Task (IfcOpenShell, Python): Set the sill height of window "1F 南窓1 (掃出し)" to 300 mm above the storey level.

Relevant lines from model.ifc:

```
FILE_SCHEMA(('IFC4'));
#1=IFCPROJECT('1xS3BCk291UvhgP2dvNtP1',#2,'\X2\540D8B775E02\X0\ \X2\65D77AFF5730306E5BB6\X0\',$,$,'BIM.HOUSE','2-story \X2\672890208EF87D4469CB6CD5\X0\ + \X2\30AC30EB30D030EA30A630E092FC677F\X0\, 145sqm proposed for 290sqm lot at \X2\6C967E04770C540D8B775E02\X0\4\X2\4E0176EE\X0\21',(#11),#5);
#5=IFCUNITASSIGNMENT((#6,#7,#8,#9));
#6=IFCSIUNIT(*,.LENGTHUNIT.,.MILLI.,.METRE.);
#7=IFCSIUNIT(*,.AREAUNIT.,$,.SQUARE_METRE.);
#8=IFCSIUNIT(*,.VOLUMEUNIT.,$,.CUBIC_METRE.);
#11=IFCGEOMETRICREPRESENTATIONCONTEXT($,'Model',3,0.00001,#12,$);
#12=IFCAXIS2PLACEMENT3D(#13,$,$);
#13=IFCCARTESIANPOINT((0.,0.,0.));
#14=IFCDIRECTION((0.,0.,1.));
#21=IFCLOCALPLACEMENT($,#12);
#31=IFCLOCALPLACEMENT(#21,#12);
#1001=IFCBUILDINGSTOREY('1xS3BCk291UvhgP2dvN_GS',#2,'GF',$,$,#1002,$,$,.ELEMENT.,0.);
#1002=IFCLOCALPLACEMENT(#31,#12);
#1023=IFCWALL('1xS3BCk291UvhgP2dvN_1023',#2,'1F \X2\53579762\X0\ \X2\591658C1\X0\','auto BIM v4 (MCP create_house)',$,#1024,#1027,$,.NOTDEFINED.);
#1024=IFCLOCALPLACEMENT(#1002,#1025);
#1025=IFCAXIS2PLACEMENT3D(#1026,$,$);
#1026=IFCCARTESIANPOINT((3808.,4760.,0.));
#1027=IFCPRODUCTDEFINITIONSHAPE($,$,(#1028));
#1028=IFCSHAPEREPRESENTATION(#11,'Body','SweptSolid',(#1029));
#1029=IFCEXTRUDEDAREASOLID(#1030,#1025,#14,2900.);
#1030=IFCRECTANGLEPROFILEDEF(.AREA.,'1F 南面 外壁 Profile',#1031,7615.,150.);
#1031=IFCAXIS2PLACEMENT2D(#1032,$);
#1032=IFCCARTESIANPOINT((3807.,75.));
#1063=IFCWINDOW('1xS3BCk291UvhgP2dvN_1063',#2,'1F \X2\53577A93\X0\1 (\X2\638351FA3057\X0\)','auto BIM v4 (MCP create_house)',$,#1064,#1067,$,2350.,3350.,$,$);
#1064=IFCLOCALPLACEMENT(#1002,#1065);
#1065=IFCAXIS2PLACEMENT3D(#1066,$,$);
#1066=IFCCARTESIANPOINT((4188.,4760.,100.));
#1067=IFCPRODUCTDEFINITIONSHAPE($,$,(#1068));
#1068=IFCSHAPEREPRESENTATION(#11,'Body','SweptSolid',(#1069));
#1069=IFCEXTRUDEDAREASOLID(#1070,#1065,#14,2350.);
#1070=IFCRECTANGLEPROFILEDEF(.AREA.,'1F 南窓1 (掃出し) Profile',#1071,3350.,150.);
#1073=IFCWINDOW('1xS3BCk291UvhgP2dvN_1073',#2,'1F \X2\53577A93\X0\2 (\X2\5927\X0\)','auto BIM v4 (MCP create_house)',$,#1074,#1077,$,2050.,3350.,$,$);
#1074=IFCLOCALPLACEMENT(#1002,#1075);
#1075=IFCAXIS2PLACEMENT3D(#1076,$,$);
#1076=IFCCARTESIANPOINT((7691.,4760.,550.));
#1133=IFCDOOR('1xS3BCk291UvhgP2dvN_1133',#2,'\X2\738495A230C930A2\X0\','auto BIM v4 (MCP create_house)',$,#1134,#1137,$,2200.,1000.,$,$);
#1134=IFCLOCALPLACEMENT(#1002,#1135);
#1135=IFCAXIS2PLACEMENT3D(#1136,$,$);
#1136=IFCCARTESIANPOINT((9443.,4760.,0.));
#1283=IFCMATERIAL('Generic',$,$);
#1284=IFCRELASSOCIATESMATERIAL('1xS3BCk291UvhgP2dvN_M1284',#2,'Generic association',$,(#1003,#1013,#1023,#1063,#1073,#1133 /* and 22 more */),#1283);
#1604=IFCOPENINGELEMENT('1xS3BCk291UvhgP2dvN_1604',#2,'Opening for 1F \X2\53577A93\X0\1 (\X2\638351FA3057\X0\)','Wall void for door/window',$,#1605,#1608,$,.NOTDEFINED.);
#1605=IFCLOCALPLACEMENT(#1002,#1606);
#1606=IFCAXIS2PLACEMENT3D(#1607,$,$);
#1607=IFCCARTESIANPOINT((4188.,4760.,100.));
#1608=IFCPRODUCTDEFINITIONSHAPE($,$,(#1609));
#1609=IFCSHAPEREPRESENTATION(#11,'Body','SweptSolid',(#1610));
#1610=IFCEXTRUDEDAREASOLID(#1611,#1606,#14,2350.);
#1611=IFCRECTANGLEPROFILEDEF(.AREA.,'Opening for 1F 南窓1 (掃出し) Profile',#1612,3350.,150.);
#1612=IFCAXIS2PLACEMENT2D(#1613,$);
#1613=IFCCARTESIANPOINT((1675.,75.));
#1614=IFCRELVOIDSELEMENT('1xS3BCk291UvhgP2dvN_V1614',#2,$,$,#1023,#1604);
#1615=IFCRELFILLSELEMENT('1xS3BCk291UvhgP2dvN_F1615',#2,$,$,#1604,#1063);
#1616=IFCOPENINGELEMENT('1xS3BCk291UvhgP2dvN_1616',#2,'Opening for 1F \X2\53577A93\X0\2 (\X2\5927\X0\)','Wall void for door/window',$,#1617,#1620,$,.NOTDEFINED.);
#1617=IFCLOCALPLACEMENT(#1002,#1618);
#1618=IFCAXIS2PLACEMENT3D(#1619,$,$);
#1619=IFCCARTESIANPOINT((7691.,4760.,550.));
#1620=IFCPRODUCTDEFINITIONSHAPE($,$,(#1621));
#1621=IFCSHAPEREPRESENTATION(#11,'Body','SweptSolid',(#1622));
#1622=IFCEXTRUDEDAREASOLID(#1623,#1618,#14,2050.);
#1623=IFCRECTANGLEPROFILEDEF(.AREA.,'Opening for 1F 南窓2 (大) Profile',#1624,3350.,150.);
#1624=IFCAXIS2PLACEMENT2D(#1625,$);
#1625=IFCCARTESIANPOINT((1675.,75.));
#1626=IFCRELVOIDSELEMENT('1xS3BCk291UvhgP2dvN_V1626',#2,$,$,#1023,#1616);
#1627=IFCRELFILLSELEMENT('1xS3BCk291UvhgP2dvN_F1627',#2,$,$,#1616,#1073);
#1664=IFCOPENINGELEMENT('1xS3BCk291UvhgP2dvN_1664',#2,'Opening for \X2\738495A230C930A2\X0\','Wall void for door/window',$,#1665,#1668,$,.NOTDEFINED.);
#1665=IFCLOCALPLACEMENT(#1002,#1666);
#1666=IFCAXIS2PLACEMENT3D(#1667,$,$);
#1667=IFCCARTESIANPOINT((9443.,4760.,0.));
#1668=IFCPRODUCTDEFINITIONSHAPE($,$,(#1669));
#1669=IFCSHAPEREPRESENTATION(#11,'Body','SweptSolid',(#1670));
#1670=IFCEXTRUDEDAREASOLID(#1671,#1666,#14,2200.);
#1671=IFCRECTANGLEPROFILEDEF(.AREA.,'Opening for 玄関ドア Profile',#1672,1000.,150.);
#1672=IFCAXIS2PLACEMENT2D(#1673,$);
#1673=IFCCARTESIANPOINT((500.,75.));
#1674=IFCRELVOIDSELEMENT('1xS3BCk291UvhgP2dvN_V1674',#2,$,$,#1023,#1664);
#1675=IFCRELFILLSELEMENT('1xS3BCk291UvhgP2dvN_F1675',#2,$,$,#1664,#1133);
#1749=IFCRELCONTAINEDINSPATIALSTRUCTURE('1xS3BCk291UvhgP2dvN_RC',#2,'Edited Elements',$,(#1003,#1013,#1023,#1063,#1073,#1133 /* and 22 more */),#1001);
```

```python
import numpy as np
import ifcopenshell
import ifcopenshell.api.geometry
import ifcopenshell.geom
import ifcopenshell.util.element
import ifcopenshell.util.placement
import ifcopenshell.util.shape
import ifcopenshell.util.unit

model = ifcopenshell.open("model.ifc")
unit_scale = ifcopenshell.util.unit.calculate_unit_scale(model)

window = model.by_guid("1xS3BCk291UvhgP2dvN_1063")
opening = window.FillsVoids[0].RelatingOpeningElement
storey = ifcopenshell.util.element.get_container(window, ifc_class="IfcBuildingStorey")
level = ifcopenshell.util.placement.get_local_placement(storey.ObjectPlacement)[2, 3]

# The opening's origin need not be at the sill, so measure its lowest point.
shape = ifcopenshell.geom.create_shape(ifcopenshell.geom.settings(), opening)
bottom = ifcopenshell.util.shape.get_shape_bottom_elevation(shape, shape.geometry) / unit_scale
dz = level + 0.3 / unit_scale - bottom

shift = np.array([0.0, 0.0, dz])
# The window is not placed relative to its opening, so move both.
for product in (opening, window):
    matrix = ifcopenshell.util.placement.get_local_placement(product.ObjectPlacement)
    matrix[:3, 3] += shift
    ifcopenshell.api.geometry.edit_object_placement(model, product=product, matrix=matrix, is_si=False)

print(f"moved by {dz * unit_scale:+.3f} m")

model.write("model_rev.ifc")
```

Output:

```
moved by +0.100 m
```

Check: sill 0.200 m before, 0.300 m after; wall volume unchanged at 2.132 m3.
